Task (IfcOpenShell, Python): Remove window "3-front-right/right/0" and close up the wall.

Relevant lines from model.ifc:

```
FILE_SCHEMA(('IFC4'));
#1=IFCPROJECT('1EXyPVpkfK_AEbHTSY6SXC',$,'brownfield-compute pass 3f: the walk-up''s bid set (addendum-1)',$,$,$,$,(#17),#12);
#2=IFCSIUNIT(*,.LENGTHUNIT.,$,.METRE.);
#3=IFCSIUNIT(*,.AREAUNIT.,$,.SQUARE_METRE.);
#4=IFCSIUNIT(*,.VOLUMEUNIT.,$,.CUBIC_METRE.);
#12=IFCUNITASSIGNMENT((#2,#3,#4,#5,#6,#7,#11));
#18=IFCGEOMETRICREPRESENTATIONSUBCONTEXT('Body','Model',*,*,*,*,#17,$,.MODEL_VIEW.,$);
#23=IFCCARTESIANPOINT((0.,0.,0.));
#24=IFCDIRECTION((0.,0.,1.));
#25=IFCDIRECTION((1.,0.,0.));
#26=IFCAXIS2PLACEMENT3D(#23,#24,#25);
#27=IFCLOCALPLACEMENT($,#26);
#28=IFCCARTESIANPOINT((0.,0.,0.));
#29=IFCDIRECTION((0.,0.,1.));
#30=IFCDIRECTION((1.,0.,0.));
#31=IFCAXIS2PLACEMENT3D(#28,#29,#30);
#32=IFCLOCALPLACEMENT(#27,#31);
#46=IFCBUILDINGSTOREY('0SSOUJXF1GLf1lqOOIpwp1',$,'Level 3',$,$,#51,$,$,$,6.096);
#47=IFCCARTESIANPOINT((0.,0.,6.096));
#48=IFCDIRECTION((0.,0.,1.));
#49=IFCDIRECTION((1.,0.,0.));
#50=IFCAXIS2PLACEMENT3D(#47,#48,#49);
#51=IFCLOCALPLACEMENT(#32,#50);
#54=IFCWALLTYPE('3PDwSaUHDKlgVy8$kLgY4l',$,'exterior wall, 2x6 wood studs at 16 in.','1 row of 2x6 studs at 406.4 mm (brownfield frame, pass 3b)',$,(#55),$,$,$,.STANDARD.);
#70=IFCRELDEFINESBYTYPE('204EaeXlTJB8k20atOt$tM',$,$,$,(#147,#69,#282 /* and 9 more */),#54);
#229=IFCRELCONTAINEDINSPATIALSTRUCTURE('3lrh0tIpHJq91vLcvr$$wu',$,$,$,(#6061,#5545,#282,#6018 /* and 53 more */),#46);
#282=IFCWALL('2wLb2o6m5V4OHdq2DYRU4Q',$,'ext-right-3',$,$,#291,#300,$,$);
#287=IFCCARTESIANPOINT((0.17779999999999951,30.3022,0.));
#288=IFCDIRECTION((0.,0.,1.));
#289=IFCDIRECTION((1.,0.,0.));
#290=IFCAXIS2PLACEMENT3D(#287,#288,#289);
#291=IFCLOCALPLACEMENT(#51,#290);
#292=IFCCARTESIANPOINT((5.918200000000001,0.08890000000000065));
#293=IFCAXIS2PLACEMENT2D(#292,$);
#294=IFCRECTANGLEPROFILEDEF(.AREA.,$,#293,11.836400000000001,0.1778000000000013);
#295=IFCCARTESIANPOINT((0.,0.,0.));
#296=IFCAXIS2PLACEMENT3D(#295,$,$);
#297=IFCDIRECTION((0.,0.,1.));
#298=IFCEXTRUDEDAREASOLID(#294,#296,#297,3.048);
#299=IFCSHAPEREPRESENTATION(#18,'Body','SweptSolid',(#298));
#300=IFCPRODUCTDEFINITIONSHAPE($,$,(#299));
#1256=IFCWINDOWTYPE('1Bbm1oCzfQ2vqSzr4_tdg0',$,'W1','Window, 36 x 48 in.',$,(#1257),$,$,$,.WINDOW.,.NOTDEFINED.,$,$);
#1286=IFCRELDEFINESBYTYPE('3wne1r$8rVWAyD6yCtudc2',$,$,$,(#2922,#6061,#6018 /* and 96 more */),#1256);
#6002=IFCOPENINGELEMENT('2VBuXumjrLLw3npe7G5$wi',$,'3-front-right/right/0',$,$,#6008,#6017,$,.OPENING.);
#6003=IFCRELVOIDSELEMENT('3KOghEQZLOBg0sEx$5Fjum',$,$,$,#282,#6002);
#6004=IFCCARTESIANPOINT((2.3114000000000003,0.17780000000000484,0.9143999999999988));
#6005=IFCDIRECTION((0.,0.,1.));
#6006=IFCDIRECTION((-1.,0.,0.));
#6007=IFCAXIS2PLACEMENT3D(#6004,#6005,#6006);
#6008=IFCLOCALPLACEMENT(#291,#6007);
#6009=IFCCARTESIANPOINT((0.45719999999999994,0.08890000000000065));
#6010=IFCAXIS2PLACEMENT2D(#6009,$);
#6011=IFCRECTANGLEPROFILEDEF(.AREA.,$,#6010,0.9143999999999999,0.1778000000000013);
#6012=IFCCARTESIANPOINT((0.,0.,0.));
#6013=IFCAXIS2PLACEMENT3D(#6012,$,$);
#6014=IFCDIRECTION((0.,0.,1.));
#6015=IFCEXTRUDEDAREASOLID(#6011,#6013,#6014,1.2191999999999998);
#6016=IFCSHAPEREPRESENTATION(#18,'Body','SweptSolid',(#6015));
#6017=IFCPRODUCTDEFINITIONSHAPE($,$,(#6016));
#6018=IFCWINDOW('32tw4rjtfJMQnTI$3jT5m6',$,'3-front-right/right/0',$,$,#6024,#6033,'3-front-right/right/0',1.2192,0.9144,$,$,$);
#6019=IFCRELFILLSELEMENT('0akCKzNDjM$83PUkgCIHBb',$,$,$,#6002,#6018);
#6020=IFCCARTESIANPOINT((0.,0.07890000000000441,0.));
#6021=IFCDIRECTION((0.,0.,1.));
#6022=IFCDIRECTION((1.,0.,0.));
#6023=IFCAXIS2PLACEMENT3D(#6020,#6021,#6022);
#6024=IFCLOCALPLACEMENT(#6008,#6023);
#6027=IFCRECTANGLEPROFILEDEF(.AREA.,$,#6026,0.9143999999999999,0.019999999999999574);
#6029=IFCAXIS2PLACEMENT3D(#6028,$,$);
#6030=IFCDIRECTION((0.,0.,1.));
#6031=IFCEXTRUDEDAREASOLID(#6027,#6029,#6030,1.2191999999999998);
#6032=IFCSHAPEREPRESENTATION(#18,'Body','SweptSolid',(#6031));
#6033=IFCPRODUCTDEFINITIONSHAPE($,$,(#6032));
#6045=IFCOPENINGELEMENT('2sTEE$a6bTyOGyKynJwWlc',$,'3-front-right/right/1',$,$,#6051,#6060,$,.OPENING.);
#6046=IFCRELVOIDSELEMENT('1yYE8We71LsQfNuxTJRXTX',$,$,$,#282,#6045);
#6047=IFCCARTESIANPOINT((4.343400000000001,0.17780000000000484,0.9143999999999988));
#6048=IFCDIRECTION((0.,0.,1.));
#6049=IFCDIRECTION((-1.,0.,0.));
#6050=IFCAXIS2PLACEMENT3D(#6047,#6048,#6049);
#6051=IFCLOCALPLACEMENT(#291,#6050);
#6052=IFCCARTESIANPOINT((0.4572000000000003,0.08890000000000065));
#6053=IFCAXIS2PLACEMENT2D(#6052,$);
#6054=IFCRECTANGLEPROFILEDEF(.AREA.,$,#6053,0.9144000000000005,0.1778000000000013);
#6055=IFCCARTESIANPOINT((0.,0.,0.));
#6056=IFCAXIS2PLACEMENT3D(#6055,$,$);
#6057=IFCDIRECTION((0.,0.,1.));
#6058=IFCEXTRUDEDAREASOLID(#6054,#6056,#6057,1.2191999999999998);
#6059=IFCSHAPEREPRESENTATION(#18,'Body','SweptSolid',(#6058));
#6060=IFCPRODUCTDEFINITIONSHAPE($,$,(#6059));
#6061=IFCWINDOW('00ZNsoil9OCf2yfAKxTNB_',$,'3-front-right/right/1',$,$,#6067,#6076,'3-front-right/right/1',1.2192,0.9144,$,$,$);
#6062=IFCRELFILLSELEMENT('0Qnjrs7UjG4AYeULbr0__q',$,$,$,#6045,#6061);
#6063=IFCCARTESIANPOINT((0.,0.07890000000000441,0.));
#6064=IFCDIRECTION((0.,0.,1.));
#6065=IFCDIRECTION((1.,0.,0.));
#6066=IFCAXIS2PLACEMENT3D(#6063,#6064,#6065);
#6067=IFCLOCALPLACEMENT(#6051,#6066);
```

```python
import ifcopenshell
import ifcopenshell.api.feature
import ifcopenshell.api.root
import ifcopenshell.geom
import ifcopenshell.util.shape

model = ifcopenshell.open("model.ifc")
settings = ifcopenshell.geom.settings()


def volume(element):
    """Net volume in cubic metres, openings subtracted."""
    shape = ifcopenshell.geom.create_shape(settings, element)
    return ifcopenshell.util.shape.get_volume(shape.geometry)


window = model.by_id(6018)
opening = window.FillsVoids[0].RelatingOpeningElement
wall = opening.VoidsElements[0].RelatingBuildingElement
before = volume(wall)

ifcopenshell.api.root.remove_product(model, product=window)
ifcopenshell.api.feature.remove_feature(model, feature=opening)

after = volume(wall)

print(f"wall volume {before:.3f} -> {after:.3f} m3")

model.write("model_v2.ifc")
```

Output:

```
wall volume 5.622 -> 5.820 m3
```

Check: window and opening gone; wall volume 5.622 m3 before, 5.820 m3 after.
